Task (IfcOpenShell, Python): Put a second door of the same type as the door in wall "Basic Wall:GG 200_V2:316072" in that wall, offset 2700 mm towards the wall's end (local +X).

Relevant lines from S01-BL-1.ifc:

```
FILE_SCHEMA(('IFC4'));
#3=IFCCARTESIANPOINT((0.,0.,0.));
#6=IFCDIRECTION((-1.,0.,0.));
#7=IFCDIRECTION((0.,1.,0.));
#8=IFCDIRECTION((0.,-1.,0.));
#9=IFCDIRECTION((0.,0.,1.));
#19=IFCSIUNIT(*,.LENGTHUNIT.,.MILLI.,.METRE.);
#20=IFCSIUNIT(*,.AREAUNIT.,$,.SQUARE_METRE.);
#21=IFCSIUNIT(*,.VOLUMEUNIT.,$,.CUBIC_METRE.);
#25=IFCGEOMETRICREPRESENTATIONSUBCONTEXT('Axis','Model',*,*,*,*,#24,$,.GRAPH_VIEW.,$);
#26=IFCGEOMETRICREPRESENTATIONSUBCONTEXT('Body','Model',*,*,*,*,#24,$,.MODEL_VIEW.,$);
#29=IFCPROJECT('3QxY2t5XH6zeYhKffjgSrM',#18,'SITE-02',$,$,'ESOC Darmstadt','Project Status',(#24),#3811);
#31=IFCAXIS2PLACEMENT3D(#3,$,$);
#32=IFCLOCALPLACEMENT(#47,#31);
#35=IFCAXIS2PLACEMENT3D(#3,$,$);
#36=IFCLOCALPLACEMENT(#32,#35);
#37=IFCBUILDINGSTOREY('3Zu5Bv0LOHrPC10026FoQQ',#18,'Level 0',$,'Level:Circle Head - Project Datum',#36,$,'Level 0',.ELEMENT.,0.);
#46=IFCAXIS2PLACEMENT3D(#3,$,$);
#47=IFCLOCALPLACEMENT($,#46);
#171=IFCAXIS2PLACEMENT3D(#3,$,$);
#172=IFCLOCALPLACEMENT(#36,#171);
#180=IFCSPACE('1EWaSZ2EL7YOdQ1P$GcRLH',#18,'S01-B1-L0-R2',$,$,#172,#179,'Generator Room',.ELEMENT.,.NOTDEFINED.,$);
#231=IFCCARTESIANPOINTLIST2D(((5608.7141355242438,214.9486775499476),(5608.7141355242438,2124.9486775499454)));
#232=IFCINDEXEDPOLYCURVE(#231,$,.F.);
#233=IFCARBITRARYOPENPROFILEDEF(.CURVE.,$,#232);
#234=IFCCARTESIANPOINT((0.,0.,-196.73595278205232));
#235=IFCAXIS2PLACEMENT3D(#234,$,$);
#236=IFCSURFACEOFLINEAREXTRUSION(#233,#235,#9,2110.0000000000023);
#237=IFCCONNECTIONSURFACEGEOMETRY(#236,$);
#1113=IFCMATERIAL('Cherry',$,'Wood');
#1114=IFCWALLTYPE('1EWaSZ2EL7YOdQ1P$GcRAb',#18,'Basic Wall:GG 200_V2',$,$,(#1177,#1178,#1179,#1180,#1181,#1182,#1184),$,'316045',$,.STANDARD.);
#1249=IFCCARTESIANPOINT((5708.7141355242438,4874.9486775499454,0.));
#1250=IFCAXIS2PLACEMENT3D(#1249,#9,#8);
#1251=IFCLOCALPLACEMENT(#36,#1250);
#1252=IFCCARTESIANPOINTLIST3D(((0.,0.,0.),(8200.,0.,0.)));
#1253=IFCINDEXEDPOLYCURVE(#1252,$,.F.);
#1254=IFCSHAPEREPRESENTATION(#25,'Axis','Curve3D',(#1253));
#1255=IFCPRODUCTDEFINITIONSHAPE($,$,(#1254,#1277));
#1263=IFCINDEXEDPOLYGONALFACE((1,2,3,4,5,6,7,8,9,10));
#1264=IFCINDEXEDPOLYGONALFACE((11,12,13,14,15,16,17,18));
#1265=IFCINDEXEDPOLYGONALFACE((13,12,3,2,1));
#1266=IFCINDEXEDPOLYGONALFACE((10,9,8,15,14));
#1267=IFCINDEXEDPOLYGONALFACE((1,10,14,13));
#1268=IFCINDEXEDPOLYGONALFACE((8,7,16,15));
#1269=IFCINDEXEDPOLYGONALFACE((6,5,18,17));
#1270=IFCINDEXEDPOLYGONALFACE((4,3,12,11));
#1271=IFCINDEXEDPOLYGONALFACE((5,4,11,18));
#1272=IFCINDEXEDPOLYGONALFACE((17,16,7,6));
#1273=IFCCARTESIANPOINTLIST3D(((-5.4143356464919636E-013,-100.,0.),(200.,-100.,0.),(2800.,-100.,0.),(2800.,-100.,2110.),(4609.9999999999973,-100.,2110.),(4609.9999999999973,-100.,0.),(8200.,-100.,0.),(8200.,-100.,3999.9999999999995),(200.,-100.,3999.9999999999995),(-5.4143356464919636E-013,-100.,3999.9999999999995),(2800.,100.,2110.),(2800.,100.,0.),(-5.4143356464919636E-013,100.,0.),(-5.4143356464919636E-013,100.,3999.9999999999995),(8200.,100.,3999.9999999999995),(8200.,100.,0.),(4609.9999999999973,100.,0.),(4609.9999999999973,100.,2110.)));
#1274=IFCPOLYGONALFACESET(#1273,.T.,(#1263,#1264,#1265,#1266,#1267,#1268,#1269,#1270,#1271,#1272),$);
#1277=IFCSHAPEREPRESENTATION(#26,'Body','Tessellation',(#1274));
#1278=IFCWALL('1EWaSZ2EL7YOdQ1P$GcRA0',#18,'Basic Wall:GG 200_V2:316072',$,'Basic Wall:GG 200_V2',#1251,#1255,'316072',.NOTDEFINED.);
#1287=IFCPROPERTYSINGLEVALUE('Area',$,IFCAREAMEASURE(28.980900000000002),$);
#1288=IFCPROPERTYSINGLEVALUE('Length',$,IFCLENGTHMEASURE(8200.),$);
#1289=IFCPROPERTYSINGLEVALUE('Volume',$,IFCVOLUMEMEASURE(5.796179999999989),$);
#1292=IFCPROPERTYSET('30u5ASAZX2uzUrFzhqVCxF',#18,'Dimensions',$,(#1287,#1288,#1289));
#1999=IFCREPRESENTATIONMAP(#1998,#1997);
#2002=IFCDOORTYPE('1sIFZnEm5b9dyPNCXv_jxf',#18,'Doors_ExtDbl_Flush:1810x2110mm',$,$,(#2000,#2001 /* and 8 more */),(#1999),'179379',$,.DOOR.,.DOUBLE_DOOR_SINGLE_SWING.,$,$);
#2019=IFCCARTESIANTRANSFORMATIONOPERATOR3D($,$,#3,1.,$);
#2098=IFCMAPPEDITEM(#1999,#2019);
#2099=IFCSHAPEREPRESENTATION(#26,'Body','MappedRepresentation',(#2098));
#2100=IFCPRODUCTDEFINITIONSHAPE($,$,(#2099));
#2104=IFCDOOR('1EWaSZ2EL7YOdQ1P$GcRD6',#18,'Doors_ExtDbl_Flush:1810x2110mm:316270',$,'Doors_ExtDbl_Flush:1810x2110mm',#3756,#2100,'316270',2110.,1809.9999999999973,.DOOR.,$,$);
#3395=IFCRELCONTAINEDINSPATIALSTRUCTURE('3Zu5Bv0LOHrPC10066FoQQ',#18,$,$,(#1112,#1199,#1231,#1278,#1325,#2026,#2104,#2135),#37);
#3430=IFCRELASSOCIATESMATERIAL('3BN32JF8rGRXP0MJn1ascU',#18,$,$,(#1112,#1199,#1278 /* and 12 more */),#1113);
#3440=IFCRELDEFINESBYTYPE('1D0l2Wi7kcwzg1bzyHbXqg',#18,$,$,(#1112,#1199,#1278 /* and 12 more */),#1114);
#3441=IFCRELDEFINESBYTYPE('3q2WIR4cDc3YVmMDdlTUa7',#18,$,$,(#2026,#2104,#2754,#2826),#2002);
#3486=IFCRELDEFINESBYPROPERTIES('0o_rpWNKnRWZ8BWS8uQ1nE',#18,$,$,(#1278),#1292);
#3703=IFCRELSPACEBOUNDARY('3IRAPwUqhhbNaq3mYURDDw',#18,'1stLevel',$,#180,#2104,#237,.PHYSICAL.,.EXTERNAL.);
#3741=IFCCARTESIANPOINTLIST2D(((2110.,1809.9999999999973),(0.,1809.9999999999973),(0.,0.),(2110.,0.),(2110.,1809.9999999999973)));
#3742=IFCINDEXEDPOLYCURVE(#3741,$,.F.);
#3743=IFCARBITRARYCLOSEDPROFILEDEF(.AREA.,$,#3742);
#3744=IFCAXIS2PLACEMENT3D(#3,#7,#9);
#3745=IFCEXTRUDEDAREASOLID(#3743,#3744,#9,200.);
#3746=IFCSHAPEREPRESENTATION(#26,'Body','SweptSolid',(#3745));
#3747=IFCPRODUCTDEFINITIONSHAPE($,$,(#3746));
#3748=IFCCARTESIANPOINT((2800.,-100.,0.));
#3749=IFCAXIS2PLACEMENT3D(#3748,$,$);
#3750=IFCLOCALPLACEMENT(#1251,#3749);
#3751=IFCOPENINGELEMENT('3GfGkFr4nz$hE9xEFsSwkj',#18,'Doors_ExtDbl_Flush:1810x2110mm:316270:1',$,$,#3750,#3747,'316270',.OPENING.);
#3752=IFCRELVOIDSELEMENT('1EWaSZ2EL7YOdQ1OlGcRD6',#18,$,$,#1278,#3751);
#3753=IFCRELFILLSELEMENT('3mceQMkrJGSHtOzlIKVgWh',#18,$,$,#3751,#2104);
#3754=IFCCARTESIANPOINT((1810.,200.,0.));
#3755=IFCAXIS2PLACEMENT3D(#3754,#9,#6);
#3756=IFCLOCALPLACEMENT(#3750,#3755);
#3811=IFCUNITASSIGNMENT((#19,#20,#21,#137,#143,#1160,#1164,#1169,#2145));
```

```python
import numpy as np
import ifcopenshell
import ifcopenshell.api.feature
import ifcopenshell.api.geometry
import ifcopenshell.api.pset
import ifcopenshell.api.root
import ifcopenshell.geom
import ifcopenshell.util.element
import ifcopenshell.util.placement
import ifcopenshell.util.shape
import ifcopenshell.util.unit

model = ifcopenshell.open("S01-BL-1.ifc")
unit_scale = ifcopenshell.util.unit.calculate_unit_scale(model)
area_scale = ifcopenshell.util.unit.calculate_unit_scale(model, "AREAUNIT")
volume_scale = ifcopenshell.util.unit.calculate_unit_scale(model, "VOLUMEUNIT")
settings = ifcopenshell.geom.settings()


def volume(element):
    """Net volume in cubic metres, openings subtracted."""
    shape = ifcopenshell.geom.create_shape(settings, element)
    return ifcopenshell.util.shape.get_volume(shape.geometry)


def reuse_history(source, copy):
    """copy_class also copies each property set's owner history, people and application; keep the originals."""
    for rel in copy.IsDefinedBy:
        if rel.is_a("IfcRelDefinesByProperties") and (history := rel.RelatingPropertyDefinition.OwnerHistory):
            rel.RelatingPropertyDefinition.OwnerHistory = source.OwnerHistory
            ifcopenshell.util.element.remove_deep2(model, history)


door = model.by_id(2104)
opening = door.FillsVoids[0].RelatingOpeningElement
wall = opening.VoidsElements[0].RelatingBuildingElement
before = volume(wall)
shift = ifcopenshell.util.placement.get_local_placement(wall.ObjectPlacement)[:3, 0] * 2.7 / unit_scale

# copy_class copies the void relationship, type, container and properties, but no geometry.
new_opening = ifcopenshell.api.root.copy_class(model, product=opening)
new_opening.Representation = ifcopenshell.util.element.copy_deep(
    model, opening.Representation, exclude=["IfcGeometricRepresentationContext", "IfcRepresentationMap"]
)
new_opening.Name = "Doors_ExtDbl_Flush:1810x2110mm"
new_opening.Tag = None
new_door = ifcopenshell.api.root.copy_class(model, product=door)
new_door.Representation = ifcopenshell.util.element.copy_deep(
    model, door.Representation, exclude=["IfcGeometricRepresentationContext", "IfcRepresentationMap"]
)
new_door.Name = "Doors_ExtDbl_Flush:1810x2110mm"
new_door.Tag = None
reuse_history(door, new_door)
ifcopenshell.api.feature.add_filling(model, opening=new_opening, element=new_door)

for old, new in ((opening, new_opening), (door, new_door)):
    matrix = ifcopenshell.util.placement.get_local_placement(old.ObjectPlacement)
    matrix[:3, 3] += shift
    ifcopenshell.api.geometry.edit_object_placement(model, product=new, matrix=matrix, is_si=False)

# The copied space boundaries still share their surfaces with the original.
for rel in new_door.ProvidesBoundaries:
    if rel.ConnectionGeometry:
        rel.ConnectionGeometry = ifcopenshell.util.element.copy_deep(model, rel.ConnectionGeometry)

# Space boundary surfaces are stored in each space's coordinates; move them too.
for rel in new_door.ProvidesBoundaries:
    if not rel.ConnectionGeometry:
        continue
    surface = rel.ConnectionGeometry.SurfaceOnRelatingElement
    space_matrix = ifcopenshell.util.placement.get_local_placement(rel.RelatingSpace.ObjectPlacement)
    point = np.array(surface.Position.Location.Coordinates) + space_matrix[:3, :3].T @ shift
    surface.Position = model.createIfcAxis2Placement3D(
        model.createIfcCartesianPoint(point.tolist()), surface.Position.Axis, surface.Position.RefDirection
    )

after = volume(wall)
thickness = 0.2  # wall thickness in metres

# Update the wall's stored quantities.
pset = model.by_id(ifcopenshell.util.element.get_pset(wall, "Dimensions", should_inherit=False)["id"])
ifcopenshell.api.pset.edit_pset(model, pset=pset, properties={
    "Area": model.create_entity("IfcAreaMeasure", after / thickness / area_scale),
    "Volume": model.create_entity("IfcVolumeMeasure", after / volume_scale),
})

print(f"wall volume {before:.3f} -> {after:.3f} m3")

model.write("S01-BL-1_v2.ifc")
```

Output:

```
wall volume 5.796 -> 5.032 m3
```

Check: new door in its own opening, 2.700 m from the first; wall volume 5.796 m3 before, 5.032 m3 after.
